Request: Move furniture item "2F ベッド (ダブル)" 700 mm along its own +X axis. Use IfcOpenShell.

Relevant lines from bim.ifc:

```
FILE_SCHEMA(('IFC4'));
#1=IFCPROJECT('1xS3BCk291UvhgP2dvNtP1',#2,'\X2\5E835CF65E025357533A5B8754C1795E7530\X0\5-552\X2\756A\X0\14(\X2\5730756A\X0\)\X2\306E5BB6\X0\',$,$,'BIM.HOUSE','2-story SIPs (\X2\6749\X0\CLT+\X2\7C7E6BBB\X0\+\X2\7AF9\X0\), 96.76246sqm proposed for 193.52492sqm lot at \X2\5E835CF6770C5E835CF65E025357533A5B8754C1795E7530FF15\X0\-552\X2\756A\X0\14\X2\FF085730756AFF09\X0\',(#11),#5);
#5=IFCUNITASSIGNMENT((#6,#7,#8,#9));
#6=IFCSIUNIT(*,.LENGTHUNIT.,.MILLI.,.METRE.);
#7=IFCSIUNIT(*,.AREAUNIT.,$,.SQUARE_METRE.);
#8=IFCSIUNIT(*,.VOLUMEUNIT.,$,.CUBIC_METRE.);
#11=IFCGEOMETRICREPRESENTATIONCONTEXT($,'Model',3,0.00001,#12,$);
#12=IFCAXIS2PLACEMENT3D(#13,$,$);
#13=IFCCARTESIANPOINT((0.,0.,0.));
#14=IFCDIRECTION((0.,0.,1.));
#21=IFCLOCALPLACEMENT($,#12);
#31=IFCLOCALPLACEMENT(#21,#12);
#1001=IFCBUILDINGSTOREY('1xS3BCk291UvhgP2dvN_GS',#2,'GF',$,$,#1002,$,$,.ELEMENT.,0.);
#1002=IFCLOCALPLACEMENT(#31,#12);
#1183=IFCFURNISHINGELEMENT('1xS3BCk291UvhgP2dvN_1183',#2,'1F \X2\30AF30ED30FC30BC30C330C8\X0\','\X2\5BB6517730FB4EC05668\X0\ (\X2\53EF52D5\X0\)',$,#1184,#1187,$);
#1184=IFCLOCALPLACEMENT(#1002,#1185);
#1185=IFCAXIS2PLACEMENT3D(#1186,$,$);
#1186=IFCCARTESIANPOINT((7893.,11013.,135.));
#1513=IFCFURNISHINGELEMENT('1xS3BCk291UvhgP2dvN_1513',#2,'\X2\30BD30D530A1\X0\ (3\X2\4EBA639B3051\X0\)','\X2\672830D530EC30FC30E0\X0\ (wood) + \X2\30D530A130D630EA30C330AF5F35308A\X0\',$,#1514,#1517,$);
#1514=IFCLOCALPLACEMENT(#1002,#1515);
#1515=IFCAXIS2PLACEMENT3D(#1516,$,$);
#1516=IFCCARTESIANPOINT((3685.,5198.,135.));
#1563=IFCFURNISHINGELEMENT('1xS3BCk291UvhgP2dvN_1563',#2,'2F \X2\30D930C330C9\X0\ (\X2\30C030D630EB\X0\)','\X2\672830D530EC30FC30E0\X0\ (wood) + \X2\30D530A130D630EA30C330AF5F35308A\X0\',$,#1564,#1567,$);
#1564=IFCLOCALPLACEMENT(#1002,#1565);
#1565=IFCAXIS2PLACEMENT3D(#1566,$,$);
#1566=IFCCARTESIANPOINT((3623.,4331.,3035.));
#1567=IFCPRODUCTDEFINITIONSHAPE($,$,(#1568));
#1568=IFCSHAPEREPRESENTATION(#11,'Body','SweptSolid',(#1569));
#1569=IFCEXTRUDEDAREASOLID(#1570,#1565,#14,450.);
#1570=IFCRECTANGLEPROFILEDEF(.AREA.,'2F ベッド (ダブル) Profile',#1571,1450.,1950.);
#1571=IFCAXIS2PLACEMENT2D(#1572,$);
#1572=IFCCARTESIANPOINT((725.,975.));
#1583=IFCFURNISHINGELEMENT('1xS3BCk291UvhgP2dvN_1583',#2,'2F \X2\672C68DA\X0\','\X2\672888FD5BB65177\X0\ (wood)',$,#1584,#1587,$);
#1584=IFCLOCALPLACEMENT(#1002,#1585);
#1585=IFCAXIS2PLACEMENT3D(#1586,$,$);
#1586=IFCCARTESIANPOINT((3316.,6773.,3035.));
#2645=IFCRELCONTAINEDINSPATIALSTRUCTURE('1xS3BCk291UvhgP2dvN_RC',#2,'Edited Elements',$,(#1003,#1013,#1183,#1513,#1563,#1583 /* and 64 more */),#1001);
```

```python
import ifcopenshell
import ifcopenshell.api.geometry
import ifcopenshell.util.placement
import ifcopenshell.util.unit

model = ifcopenshell.open("bim.ifc")
unit_scale = ifcopenshell.util.unit.calculate_unit_scale(model)

item = model.by_guid("1xS3BCk291UvhgP2dvN_1563")
matrix = ifcopenshell.util.placement.get_local_placement(item.ObjectPlacement)
matrix[:3, 3] += matrix[:3, 0] * 0.7 / unit_scale
ifcopenshell.api.geometry.edit_object_placement(model, product=item, matrix=matrix, is_si=False)

print(ifcopenshell.util.placement.get_local_placement(item.ObjectPlacement).round(3) + 0.0)

model.write("bim_v2.ifc")
```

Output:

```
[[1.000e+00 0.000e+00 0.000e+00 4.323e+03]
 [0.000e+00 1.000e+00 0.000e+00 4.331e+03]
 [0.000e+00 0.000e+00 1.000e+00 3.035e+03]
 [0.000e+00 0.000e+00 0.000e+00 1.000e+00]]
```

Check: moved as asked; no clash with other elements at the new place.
